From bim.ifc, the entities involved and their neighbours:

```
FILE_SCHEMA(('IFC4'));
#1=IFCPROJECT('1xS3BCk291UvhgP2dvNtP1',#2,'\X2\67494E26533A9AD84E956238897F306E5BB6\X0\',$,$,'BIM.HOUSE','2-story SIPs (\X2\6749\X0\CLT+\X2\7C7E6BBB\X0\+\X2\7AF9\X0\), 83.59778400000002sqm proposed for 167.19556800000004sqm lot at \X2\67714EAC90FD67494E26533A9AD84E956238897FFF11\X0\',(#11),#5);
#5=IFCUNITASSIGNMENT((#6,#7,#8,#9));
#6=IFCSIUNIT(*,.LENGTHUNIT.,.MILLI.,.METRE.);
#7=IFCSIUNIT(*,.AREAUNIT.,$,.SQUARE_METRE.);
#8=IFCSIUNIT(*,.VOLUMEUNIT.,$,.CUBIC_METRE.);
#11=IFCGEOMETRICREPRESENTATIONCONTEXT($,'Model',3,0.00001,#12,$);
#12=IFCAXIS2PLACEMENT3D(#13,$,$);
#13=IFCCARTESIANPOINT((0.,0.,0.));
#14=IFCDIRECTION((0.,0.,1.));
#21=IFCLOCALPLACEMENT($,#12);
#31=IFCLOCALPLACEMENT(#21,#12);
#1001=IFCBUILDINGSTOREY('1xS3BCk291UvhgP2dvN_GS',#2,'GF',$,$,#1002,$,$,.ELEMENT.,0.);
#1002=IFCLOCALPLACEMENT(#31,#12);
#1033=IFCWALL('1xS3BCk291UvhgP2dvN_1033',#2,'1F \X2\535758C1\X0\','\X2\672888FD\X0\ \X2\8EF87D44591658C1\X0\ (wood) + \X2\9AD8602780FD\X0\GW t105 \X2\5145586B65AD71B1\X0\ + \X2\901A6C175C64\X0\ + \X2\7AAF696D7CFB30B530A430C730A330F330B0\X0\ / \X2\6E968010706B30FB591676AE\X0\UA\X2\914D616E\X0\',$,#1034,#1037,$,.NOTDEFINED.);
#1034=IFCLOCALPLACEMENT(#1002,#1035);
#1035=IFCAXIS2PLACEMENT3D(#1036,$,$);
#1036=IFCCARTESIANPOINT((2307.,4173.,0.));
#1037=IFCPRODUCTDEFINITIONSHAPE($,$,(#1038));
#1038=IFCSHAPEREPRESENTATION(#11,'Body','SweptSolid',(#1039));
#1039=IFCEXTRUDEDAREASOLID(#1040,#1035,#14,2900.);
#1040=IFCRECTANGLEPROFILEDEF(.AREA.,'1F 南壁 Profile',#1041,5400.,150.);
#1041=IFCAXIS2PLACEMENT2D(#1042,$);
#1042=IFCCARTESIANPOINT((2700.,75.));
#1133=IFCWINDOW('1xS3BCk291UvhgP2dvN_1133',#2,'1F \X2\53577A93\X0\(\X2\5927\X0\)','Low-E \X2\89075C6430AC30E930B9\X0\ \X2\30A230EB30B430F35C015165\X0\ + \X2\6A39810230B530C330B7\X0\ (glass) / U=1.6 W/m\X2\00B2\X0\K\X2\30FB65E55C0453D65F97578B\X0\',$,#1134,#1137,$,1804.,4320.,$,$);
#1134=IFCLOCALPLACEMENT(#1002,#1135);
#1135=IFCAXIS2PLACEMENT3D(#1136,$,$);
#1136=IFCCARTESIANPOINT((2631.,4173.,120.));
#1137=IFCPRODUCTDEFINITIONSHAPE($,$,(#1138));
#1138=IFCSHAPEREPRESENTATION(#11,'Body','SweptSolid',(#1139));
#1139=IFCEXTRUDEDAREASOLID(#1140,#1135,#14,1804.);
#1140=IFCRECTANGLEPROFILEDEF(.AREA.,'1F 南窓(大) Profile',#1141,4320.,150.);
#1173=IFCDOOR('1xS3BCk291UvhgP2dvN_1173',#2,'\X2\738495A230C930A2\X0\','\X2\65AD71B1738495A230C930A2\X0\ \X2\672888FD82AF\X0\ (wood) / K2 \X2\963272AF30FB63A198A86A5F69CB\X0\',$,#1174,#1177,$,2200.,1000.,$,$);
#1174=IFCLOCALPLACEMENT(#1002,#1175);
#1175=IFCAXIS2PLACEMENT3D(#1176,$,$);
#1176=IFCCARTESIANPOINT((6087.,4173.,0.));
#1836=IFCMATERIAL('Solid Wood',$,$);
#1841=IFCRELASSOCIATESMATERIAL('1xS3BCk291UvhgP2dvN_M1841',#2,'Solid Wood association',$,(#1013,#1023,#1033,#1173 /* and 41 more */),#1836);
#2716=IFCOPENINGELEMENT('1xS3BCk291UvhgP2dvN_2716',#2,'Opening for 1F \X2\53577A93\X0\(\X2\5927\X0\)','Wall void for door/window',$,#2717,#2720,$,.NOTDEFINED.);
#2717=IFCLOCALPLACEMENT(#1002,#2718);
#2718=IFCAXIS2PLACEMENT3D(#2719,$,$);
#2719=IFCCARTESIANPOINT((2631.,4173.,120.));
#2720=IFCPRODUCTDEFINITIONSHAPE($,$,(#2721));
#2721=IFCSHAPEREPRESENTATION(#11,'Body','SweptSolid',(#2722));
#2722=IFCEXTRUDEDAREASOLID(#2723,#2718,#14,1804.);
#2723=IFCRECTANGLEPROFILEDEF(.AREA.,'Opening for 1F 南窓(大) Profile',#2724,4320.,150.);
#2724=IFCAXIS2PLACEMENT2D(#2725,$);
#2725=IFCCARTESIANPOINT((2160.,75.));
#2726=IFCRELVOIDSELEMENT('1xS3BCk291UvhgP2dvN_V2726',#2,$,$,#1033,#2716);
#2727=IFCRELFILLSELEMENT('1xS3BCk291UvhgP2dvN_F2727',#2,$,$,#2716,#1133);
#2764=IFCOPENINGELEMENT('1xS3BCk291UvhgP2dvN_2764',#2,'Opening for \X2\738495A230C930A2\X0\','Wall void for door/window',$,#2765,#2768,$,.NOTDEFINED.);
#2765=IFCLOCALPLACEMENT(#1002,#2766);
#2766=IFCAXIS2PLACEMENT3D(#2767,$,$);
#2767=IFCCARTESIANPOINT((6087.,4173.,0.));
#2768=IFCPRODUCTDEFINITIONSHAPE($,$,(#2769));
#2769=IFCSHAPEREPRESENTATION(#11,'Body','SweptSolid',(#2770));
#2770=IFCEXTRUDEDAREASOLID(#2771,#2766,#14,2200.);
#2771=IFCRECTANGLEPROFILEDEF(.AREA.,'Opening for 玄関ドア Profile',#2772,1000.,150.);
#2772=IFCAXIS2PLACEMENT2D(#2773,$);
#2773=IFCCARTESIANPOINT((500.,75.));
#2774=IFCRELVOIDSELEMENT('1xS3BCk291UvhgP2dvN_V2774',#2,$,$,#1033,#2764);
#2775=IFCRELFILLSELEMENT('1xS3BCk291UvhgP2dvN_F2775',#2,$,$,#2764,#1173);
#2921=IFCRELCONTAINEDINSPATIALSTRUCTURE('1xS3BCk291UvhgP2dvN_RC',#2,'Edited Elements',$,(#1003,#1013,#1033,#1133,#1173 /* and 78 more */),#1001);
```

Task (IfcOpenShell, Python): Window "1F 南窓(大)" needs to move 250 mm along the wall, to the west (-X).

```python
import ifcopenshell
import ifcopenshell.api.geometry
import ifcopenshell.util.placement
import ifcopenshell.util.unit

model = ifcopenshell.open("bim.ifc")
unit_scale = ifcopenshell.util.unit.calculate_unit_scale(model)

window = model.by_guid("1xS3BCk291UvhgP2dvN_1133")
opening = window.FillsVoids[0].RelatingOpeningElement
wall = opening.VoidsElements[0].RelatingBuildingElement

wall_matrix = ifcopenshell.util.placement.get_local_placement(wall.ObjectPlacement)
shift = wall_matrix[:3, 0] * -0.25 / unit_scale
before = ifcopenshell.util.placement.get_local_placement(window.ObjectPlacement)[:3, 3].copy()

# The window is not placed relative to its opening, so move both.
for product in (opening, window):
    matrix = ifcopenshell.util.placement.get_local_placement(product.ObjectPlacement)
    matrix[:3, 3] += shift
    ifcopenshell.api.geometry.edit_object_placement(model, product=product, matrix=matrix, is_si=False)

after = ifcopenshell.util.placement.get_local_placement(window.ObjectPlacement)[:3, 3]
print("window moved by", (after - before).round(3) + 0.0)

model.write("bim_rev.ifc")
```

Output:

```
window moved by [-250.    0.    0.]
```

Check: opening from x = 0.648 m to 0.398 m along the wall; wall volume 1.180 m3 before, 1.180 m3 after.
